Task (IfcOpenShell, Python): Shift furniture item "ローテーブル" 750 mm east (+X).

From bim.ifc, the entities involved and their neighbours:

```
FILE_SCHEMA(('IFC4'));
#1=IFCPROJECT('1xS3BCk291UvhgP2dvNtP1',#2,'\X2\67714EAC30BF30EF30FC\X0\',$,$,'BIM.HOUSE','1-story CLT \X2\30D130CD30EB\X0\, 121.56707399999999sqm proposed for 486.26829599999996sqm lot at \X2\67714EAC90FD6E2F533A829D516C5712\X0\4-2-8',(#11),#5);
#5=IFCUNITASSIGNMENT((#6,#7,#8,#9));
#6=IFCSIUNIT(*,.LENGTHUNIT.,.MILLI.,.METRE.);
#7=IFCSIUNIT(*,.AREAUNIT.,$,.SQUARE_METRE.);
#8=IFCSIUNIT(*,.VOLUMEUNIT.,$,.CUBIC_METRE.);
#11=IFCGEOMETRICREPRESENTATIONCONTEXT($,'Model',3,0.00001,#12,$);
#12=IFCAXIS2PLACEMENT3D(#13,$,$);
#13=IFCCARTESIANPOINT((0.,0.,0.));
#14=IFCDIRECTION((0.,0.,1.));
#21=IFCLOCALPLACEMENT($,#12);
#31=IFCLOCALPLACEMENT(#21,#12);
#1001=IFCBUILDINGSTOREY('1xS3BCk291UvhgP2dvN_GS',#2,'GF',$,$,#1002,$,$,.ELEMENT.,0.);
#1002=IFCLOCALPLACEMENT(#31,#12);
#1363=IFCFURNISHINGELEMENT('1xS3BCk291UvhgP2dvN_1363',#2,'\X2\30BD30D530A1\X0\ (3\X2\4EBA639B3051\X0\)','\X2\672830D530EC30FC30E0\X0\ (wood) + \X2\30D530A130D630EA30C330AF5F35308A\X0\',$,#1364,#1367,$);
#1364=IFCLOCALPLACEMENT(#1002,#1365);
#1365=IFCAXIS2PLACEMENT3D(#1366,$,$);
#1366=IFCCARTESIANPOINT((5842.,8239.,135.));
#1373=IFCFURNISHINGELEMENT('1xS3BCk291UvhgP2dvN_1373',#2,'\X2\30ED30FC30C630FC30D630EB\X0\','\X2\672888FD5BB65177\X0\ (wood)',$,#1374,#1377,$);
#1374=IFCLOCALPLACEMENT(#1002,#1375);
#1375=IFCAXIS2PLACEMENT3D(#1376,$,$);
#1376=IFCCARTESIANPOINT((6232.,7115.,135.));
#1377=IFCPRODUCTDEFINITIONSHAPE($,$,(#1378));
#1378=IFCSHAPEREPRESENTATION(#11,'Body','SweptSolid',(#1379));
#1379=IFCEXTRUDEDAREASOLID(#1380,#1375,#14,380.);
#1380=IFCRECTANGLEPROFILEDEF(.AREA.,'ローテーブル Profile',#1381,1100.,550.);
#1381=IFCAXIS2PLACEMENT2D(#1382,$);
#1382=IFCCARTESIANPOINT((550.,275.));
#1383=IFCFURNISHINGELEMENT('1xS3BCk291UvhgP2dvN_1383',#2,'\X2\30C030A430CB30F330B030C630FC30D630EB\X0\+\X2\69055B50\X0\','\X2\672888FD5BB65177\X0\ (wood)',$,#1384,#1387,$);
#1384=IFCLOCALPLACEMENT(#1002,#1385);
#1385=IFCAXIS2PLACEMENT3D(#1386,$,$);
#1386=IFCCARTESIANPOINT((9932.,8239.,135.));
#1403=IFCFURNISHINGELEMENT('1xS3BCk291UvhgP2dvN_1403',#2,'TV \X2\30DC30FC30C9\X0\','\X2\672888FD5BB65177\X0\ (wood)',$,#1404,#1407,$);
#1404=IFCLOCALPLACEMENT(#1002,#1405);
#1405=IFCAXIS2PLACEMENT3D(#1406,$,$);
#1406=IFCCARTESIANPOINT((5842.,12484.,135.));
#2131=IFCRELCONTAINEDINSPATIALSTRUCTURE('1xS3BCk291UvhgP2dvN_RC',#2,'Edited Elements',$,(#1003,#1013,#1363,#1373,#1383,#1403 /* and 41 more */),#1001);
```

```python
import ifcopenshell
import ifcopenshell.api.geometry
import ifcopenshell.util.placement
import ifcopenshell.util.unit

model = ifcopenshell.open("bim.ifc")
unit_scale = ifcopenshell.util.unit.calculate_unit_scale(model)

item = model.by_guid("1xS3BCk291UvhgP2dvN_1373")
matrix = ifcopenshell.util.placement.get_local_placement(item.ObjectPlacement)
matrix[0, 3] += 0.75 / unit_scale
ifcopenshell.api.geometry.edit_object_placement(model, product=item, matrix=matrix, is_si=False)

print(ifcopenshell.util.placement.get_local_placement(item.ObjectPlacement).round(3) + 0.0)

model.write("bim_updated.ifc")
```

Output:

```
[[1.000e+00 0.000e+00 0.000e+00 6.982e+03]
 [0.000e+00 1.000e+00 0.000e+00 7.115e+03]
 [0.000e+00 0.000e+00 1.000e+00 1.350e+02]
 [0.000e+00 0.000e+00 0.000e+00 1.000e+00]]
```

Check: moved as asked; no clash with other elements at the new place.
